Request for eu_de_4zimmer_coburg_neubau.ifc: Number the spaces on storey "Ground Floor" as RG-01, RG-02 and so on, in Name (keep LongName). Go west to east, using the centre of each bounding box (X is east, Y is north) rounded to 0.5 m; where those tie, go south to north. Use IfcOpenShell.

First a look at what the model holds.

```python
import ifcopenshell
import ifcopenshell.util.element
import ifcopenshell.util.placement

model = ifcopenshell.open("eu_de_4zimmer_coburg_neubau.ifc")
print(model.schema)
storey = next(s for s in model.by_type("IfcBuildingStorey") if s.Name == "Ground Floor")
spaces = [e for e in ifcopenshell.util.element.get_decomposition(storey) if e.is_a("IfcSpace")]
for e in sorted(spaces, key=lambda e: e.id()):
    origin = ifcopenshell.util.placement.get_local_placement(e.ObjectPlacement)[:3, 3]
    print(e.id(), e.Name, e.LongName, origin.round(2) + 0.0, sep=" | ")
```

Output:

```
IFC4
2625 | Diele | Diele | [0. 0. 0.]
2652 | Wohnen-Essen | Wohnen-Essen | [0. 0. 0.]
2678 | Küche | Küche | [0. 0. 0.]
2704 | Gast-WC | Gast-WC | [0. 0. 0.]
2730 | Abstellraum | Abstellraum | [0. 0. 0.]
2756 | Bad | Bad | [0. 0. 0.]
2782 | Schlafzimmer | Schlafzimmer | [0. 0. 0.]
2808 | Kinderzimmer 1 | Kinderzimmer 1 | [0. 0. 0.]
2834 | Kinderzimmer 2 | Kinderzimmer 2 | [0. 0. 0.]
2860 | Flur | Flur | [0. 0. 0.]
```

```python
import ifcopenshell
import ifcopenshell.geom
import ifcopenshell.util.element
import ifcopenshell.util.shape

model = ifcopenshell.open("eu_de_4zimmer_coburg_neubau.ifc")
settings = ifcopenshell.geom.settings()
settings.set("use-world-coords", True)


def centre(element):
    shape = ifcopenshell.geom.create_shape(settings, element)
    return ifcopenshell.util.shape.get_bbox_centroid(shape.geometry)


storey = next(s for s in model.by_type("IfcBuildingStorey") if s.Name == "Ground Floor")
spaces = [e for e in ifcopenshell.util.element.get_decomposition(storey) if e.is_a("IfcSpace")]

# Insertion points can sit at a corner or the storey origin, so sort by the geometry (in metres).
centres = {e: centre(e) for e in spaces}
spaces.sort(key=lambda e: (round(centres[e][0] / 0.5), centres[e][1]))

for i, e in enumerate(spaces, start=1):
    number = f"RG-{i:02d}"
    e.Name = number
    print(e.id(), number)

model.write("eu_de_4zimmer_coburg_neubau_rev.ifc")
```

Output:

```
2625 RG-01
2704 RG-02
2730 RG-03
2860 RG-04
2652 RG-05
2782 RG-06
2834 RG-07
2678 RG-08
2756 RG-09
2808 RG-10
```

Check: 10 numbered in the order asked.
